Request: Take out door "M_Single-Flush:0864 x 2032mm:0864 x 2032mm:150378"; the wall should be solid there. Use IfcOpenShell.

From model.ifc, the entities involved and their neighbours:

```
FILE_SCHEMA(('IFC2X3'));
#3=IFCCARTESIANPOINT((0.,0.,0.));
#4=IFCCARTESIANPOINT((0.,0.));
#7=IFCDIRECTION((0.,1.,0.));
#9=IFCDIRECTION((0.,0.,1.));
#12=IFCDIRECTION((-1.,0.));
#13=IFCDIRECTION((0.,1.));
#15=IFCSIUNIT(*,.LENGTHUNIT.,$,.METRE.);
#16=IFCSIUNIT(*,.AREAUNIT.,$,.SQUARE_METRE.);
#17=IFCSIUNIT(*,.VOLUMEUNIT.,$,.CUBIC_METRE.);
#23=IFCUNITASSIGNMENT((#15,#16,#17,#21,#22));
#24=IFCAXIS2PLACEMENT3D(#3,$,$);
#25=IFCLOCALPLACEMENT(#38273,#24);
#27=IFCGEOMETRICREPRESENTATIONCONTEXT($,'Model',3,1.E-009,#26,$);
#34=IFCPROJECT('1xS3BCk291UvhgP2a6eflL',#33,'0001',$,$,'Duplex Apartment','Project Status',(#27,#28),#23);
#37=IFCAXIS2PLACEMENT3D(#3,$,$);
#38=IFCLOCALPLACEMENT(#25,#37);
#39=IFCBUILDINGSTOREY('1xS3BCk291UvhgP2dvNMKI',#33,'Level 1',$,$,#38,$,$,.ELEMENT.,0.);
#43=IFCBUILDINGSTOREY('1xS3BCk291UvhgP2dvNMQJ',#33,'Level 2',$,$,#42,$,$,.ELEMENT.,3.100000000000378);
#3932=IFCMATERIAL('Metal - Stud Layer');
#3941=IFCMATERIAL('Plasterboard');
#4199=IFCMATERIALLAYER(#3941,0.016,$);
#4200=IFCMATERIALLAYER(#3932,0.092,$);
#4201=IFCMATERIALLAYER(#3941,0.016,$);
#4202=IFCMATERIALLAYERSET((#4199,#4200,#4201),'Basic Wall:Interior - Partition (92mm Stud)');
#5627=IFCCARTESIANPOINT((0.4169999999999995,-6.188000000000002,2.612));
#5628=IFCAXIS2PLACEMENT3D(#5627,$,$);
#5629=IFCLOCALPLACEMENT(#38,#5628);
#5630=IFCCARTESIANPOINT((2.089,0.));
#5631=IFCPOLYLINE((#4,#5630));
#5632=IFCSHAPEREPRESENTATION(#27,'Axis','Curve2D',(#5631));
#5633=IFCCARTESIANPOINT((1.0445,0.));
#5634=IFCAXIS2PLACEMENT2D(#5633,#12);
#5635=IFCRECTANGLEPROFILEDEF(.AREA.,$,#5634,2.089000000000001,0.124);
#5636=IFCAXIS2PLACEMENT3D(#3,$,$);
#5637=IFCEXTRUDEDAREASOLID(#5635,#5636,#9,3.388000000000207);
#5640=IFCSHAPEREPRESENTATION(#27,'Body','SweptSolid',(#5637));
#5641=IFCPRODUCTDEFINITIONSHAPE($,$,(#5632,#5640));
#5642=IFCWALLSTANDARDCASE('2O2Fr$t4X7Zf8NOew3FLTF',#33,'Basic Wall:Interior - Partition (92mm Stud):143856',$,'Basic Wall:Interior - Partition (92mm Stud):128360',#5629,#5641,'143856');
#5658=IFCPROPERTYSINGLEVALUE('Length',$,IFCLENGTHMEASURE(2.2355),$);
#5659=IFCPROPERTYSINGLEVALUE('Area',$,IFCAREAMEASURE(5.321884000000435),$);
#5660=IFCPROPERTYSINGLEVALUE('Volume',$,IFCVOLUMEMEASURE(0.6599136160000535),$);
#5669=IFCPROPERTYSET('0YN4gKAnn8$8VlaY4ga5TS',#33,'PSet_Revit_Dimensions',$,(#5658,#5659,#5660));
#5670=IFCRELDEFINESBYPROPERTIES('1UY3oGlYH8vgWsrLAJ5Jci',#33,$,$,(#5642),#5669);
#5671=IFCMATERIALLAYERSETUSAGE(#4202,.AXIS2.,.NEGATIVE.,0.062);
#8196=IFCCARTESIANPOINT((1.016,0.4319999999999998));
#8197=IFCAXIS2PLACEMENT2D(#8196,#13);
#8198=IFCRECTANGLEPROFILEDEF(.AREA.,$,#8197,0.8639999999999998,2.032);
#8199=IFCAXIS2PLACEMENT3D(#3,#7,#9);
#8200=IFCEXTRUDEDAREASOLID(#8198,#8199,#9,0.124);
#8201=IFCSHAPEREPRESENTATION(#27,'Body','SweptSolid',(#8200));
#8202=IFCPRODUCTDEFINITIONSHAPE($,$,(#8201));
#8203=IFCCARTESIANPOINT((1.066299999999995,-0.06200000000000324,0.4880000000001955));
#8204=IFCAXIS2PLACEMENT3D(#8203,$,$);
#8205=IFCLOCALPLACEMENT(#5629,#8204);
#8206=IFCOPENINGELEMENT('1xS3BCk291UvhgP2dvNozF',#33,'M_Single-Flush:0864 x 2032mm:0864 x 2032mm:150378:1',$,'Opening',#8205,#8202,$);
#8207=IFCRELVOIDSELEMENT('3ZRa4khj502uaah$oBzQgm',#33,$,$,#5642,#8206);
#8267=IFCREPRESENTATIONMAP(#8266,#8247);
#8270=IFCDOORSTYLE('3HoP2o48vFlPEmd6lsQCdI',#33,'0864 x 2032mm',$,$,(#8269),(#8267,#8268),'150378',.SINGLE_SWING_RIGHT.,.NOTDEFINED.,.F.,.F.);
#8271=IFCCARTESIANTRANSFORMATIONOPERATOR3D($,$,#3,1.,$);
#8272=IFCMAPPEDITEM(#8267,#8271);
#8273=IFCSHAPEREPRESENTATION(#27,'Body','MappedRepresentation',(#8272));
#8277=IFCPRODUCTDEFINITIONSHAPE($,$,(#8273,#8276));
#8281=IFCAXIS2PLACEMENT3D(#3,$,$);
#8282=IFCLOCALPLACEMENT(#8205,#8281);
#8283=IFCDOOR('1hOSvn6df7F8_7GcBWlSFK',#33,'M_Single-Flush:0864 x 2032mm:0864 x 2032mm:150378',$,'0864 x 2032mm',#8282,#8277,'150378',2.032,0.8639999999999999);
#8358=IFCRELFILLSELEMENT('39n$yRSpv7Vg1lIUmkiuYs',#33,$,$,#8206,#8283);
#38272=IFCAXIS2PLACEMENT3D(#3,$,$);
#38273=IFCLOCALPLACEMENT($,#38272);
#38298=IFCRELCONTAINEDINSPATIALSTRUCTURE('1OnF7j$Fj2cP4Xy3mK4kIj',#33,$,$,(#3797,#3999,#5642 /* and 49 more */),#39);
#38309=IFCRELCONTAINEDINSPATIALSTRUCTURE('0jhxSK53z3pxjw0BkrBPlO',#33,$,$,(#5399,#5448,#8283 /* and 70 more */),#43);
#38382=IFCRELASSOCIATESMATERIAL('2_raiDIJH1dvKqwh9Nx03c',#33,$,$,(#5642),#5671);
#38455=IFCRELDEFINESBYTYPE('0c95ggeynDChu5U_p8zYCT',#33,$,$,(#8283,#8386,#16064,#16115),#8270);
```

```python
import ifcopenshell
import ifcopenshell.api.feature
import ifcopenshell.api.pset
import ifcopenshell.api.root
import ifcopenshell.geom
import ifcopenshell.util.element
import ifcopenshell.util.shape
import ifcopenshell.util.unit

model = ifcopenshell.open("model.ifc")
area_scale = ifcopenshell.util.unit.calculate_unit_scale(model, "AREAUNIT")
volume_scale = ifcopenshell.util.unit.calculate_unit_scale(model, "VOLUMEUNIT")
settings = ifcopenshell.geom.settings()


def volume(element):
    """Net volume in cubic metres, openings subtracted."""
    shape = ifcopenshell.geom.create_shape(settings, element)
    return ifcopenshell.util.shape.get_volume(shape.geometry)


door = model.by_guid("1hOSvn6df7F8_7GcBWlSFK")
opening = door.FillsVoids[0].RelatingOpeningElement
wall = opening.VoidsElements[0].RelatingBuildingElement
before = volume(wall)

ifcopenshell.api.root.remove_product(model, product=door)
ifcopenshell.api.feature.remove_feature(model, feature=opening)

after = volume(wall)
thickness = 0.124  # wall thickness in metres

# Update the wall's stored quantities.
pset = model.by_id(ifcopenshell.util.element.get_pset(wall, "PSet_Revit_Dimensions", should_inherit=False)["id"])
ifcopenshell.api.pset.edit_pset(model, pset=pset, properties={
    "Area": model.create_entity("IfcAreaMeasure", after / thickness / area_scale),
    "Volume": model.create_entity("IfcVolumeMeasure", after / volume_scale),
})

print(f"wall volume {before:.3f} -> {after:.3f} m3")

model.write("model_edited.ifc")
```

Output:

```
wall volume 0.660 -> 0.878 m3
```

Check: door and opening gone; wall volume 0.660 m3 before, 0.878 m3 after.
